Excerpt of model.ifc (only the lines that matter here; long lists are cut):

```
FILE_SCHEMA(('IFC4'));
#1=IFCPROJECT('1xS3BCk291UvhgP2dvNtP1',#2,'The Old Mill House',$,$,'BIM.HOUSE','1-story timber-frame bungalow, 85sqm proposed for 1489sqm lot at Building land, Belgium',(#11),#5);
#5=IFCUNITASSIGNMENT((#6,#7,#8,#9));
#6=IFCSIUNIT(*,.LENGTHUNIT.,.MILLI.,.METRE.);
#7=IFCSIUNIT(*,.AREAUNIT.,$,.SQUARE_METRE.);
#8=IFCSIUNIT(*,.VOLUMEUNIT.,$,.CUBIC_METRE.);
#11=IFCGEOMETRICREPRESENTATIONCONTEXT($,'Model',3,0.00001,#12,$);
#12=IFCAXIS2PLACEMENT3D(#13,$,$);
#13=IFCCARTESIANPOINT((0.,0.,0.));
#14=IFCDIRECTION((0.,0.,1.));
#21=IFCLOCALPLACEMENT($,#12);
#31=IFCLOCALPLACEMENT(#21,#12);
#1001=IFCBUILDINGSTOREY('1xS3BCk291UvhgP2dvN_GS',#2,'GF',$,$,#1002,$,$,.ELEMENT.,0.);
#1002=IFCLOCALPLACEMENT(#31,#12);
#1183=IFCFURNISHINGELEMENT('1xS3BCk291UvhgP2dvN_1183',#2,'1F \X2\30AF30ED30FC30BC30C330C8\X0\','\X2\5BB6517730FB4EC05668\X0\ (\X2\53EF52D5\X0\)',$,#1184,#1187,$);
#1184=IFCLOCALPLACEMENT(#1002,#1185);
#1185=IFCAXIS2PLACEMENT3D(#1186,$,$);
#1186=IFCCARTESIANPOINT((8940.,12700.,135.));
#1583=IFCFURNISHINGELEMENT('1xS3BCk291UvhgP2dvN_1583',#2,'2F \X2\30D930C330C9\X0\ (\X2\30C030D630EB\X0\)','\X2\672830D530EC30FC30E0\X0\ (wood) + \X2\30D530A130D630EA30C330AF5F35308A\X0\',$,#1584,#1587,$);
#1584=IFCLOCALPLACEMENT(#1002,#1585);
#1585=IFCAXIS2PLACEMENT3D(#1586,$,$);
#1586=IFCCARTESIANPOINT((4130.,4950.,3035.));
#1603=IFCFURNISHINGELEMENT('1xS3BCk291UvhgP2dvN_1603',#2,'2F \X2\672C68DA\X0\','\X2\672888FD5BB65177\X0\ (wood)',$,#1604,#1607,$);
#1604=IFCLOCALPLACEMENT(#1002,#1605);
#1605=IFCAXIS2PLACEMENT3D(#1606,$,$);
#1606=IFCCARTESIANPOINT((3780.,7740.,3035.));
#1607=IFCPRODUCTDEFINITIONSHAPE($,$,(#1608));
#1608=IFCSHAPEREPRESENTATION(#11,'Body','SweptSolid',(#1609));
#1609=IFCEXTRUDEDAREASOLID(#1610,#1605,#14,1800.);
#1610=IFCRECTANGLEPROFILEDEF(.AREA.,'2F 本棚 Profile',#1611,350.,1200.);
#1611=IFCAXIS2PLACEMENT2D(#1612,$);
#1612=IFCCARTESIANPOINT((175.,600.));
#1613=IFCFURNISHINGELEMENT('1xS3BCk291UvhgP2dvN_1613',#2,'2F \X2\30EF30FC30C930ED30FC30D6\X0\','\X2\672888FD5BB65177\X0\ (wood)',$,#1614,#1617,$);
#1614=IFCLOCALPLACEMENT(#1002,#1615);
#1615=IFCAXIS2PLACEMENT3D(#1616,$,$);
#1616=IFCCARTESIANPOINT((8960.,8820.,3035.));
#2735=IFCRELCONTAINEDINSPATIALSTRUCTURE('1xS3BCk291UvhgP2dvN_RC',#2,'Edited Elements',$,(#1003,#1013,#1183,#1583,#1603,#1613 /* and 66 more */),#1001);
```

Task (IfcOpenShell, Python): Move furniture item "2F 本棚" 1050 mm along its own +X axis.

```python
import ifcopenshell
import ifcopenshell.api.geometry
import ifcopenshell.util.placement
import ifcopenshell.util.unit

model = ifcopenshell.open("model.ifc")
unit_scale = ifcopenshell.util.unit.calculate_unit_scale(model)

item = model.by_guid("1xS3BCk291UvhgP2dvN_1603")
matrix = ifcopenshell.util.placement.get_local_placement(item.ObjectPlacement)
matrix[:3, 3] += matrix[:3, 0] * 1.05 / unit_scale
ifcopenshell.api.geometry.edit_object_placement(model, product=item, matrix=matrix, is_si=False)

print(ifcopenshell.util.placement.get_local_placement(item.ObjectPlacement).round(3) + 0.0)

model.write("model_updated.ifc")
```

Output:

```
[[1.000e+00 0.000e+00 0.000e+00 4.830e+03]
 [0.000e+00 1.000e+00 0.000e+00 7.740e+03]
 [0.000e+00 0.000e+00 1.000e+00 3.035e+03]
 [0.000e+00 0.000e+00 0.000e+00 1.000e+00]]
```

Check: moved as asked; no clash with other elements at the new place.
